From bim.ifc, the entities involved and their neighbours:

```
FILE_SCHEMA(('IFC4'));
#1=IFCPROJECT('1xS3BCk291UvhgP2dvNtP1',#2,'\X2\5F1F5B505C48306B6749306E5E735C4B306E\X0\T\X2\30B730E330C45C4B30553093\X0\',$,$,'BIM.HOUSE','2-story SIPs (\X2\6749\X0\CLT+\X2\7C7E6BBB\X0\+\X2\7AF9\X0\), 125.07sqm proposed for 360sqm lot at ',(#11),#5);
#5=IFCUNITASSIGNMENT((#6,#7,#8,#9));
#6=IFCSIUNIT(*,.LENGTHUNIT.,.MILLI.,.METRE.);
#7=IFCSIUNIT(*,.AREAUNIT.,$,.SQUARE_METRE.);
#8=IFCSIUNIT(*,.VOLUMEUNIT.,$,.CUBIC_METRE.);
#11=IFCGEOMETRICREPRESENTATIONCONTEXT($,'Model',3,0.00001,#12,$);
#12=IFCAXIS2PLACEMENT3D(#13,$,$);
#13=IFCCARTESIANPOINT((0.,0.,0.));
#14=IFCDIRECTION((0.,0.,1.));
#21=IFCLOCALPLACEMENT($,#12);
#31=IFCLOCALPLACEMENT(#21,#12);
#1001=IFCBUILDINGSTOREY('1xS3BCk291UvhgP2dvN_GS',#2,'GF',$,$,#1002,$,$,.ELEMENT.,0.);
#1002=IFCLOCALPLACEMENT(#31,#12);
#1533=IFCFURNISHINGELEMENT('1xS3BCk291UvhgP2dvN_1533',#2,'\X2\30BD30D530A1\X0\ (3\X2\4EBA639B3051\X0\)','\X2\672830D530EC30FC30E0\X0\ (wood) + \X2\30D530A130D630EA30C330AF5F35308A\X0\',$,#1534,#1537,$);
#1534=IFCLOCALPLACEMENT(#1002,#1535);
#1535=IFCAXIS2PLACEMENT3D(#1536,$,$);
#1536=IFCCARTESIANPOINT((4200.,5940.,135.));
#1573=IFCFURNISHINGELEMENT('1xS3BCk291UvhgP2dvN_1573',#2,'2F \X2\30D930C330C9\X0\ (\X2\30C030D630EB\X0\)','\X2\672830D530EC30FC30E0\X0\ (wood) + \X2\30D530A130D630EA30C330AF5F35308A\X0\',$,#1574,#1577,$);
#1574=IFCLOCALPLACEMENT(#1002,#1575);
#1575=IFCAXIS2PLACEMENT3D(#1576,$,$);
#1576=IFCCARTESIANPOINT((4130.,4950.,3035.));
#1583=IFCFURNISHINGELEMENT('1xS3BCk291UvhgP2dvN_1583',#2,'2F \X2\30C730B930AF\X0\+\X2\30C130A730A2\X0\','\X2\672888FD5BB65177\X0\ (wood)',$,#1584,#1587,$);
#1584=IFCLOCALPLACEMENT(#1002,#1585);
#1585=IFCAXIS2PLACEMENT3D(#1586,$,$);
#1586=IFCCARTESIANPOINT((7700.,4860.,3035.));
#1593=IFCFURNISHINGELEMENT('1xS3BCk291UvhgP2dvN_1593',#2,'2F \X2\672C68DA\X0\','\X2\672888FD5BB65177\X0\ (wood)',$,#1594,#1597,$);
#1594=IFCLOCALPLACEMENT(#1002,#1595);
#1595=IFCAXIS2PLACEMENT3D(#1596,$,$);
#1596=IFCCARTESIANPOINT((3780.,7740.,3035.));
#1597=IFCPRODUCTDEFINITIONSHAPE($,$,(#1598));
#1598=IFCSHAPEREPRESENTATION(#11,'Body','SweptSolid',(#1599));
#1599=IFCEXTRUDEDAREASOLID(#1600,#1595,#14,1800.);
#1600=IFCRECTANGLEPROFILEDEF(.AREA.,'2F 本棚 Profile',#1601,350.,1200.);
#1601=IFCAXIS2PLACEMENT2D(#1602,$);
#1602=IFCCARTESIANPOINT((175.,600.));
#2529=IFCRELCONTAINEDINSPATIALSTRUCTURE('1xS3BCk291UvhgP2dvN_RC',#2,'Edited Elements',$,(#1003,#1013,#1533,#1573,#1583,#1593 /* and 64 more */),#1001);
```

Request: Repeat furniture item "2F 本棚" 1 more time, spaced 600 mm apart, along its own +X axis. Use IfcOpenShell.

```python
import ifcopenshell
import ifcopenshell.api.geometry
import ifcopenshell.api.root
import ifcopenshell.util.element
import ifcopenshell.util.placement
import ifcopenshell.util.unit

model = ifcopenshell.open("bim.ifc")
unit_scale = ifcopenshell.util.unit.calculate_unit_scale(model)


def reuse_history(source, copy):
    """copy_class also copies each property set's owner history, people and application; keep the originals."""
    for rel in copy.IsDefinedBy:
        if rel.is_a("IfcRelDefinesByProperties") and (history := rel.RelatingPropertyDefinition.OwnerHistory):
            rel.RelatingPropertyDefinition.OwnerHistory = source.OwnerHistory
            ifcopenshell.util.element.remove_deep2(model, history)


source = model.by_guid("1xS3BCk291UvhgP2dvN_1593")
base = ifcopenshell.util.placement.get_local_placement(source.ObjectPlacement)
step = base[:3, 0] * 0.6 / unit_scale

for i in range(1, 2):
    copy = ifcopenshell.api.root.copy_class(model, product=source)
    copy.Representation = ifcopenshell.util.element.copy_deep(
        model, source.Representation, exclude=["IfcGeometricRepresentationContext", "IfcRepresentationMap"]
    )
    reuse_history(source, copy)
    matrix = base.copy()
    matrix[:3, 3] += i * step
    print("added at", matrix[:3, 3].round(3) + 0.0)
    ifcopenshell.api.geometry.edit_object_placement(model, product=copy, matrix=matrix, is_si=False)

model.write("bim_updated.ifc")
```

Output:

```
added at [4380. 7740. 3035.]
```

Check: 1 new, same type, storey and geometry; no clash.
